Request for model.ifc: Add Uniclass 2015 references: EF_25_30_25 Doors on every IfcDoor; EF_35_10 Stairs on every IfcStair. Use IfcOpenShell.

First a look at what the model holds.

```python
import ifcopenshell

model = ifcopenshell.open("model.ifc")
print(model.schema)
print("classifications:", [c.Name for c in model.by_type("IfcClassification")])
for ifc_class in ("IfcDoor", "IfcRoof", "IfcStair", "IfcWall", "IfcWindow"):
    print(ifc_class, len(model.by_type(ifc_class)))
```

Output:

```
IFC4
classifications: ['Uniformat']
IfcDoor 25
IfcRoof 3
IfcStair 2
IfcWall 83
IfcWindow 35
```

```python
import ifcopenshell
import ifcopenshell.api.classification

model = ifcopenshell.open("model.ifc")

system = ifcopenshell.api.classification.add_classification(model, classification="Uniclass 2015")

codes = {
    "IfcDoor": ("EF_25_30_25", "Doors"),
    "IfcStair": ("EF_35_10", "Stairs"),
}
for ifc_class, (code, name) in codes.items():
    products = model.by_type(ifc_class)
    ifcopenshell.api.classification.add_reference(
        model, products=products, classification=system, identification=code, name=name
    )
    print(code, len(products))

model.write("model-out.ifc")
```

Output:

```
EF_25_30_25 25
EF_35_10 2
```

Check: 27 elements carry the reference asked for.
